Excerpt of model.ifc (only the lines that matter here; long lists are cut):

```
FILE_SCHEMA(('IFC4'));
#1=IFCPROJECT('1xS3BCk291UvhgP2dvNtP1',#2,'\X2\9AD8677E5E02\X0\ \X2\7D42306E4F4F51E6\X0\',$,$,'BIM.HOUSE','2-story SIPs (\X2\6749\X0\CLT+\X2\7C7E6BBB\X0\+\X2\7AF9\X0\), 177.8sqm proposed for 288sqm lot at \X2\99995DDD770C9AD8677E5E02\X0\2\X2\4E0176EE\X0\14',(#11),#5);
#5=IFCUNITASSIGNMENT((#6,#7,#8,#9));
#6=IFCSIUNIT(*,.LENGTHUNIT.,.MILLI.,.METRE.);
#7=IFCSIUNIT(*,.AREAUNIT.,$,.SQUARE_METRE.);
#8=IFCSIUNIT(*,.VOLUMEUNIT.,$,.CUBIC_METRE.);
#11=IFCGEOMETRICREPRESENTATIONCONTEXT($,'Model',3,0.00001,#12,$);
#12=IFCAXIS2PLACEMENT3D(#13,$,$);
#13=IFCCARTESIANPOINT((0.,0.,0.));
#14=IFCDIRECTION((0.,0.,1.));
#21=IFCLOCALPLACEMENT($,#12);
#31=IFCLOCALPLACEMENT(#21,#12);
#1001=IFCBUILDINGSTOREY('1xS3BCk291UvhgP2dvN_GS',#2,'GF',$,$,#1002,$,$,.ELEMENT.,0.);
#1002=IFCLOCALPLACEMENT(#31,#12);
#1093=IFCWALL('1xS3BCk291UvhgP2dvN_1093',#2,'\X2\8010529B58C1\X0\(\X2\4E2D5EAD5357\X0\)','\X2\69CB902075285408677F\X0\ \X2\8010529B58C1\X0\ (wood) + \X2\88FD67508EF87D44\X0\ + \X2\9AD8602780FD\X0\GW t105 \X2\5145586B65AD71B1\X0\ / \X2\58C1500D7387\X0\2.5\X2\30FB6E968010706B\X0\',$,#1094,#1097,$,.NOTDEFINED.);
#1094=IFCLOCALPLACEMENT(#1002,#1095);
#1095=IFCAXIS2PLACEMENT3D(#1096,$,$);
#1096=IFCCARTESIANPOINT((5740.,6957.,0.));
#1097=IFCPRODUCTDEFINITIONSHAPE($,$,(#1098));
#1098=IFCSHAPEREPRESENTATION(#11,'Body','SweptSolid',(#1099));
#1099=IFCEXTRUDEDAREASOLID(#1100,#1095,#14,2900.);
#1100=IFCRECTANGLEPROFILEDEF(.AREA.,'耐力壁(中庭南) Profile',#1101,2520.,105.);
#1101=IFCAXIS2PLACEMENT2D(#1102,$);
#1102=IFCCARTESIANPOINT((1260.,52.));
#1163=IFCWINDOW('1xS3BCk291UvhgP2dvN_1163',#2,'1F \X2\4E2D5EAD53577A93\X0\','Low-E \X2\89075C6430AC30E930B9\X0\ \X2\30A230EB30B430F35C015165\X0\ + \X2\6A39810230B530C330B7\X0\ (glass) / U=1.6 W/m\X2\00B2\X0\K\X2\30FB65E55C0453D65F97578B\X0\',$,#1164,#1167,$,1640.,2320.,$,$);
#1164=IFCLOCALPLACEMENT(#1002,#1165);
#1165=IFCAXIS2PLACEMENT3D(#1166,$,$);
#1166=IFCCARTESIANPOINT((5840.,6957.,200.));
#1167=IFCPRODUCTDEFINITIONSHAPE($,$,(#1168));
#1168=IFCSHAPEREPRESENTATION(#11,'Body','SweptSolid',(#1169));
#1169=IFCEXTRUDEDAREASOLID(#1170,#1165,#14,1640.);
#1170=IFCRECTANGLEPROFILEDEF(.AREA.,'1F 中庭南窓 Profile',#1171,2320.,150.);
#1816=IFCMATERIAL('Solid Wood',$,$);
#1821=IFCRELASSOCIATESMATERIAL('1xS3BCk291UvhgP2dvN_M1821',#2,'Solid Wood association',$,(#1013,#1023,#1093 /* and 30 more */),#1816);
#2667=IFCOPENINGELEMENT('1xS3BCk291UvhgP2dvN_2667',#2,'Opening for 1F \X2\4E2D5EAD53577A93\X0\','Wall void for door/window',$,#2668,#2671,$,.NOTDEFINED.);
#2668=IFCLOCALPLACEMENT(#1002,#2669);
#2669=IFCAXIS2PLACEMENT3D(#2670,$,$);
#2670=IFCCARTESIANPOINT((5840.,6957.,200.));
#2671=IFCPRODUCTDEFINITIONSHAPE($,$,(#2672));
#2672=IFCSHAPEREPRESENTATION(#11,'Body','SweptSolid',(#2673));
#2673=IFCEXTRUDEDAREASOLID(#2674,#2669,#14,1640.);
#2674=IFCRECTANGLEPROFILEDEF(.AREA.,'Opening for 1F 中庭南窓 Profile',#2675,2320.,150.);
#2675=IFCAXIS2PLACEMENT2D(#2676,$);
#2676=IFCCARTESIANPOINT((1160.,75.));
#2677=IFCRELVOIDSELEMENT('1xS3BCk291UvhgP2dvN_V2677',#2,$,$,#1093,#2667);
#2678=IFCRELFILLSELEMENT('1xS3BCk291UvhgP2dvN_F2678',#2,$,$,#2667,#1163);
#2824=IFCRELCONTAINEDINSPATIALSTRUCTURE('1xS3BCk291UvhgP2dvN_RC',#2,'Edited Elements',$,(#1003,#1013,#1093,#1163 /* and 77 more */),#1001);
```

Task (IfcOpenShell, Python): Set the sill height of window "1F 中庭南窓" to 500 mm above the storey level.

```python
import numpy as np
import ifcopenshell
import ifcopenshell.api.geometry
import ifcopenshell.geom
import ifcopenshell.util.element
import ifcopenshell.util.placement
import ifcopenshell.util.shape
import ifcopenshell.util.unit

model = ifcopenshell.open("model.ifc")
unit_scale = ifcopenshell.util.unit.calculate_unit_scale(model)

window = model.by_id(1163)
opening = window.FillsVoids[0].RelatingOpeningElement
storey = ifcopenshell.util.element.get_container(window, ifc_class="IfcBuildingStorey")
level = ifcopenshell.util.placement.get_local_placement(storey.ObjectPlacement)[2, 3]

# The opening's origin need not be at the sill, so measure its lowest point.
shape = ifcopenshell.geom.create_shape(ifcopenshell.geom.settings(), opening)
bottom = ifcopenshell.util.shape.get_shape_bottom_elevation(shape, shape.geometry) / unit_scale
dz = level + 0.5 / unit_scale - bottom

shift = np.array([0.0, 0.0, dz])
# The window is not placed relative to its opening, so move both.
for product in (opening, window):
    matrix = ifcopenshell.util.placement.get_local_placement(product.ObjectPlacement)
    matrix[:3, 3] += shift
    ifcopenshell.api.geometry.edit_object_placement(model, product=product, matrix=matrix, is_si=False)

print(f"moved by {dz * unit_scale:+.3f} m")

model.write("model_rev.ifc")
```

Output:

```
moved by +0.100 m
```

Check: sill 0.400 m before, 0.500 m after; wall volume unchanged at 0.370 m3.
